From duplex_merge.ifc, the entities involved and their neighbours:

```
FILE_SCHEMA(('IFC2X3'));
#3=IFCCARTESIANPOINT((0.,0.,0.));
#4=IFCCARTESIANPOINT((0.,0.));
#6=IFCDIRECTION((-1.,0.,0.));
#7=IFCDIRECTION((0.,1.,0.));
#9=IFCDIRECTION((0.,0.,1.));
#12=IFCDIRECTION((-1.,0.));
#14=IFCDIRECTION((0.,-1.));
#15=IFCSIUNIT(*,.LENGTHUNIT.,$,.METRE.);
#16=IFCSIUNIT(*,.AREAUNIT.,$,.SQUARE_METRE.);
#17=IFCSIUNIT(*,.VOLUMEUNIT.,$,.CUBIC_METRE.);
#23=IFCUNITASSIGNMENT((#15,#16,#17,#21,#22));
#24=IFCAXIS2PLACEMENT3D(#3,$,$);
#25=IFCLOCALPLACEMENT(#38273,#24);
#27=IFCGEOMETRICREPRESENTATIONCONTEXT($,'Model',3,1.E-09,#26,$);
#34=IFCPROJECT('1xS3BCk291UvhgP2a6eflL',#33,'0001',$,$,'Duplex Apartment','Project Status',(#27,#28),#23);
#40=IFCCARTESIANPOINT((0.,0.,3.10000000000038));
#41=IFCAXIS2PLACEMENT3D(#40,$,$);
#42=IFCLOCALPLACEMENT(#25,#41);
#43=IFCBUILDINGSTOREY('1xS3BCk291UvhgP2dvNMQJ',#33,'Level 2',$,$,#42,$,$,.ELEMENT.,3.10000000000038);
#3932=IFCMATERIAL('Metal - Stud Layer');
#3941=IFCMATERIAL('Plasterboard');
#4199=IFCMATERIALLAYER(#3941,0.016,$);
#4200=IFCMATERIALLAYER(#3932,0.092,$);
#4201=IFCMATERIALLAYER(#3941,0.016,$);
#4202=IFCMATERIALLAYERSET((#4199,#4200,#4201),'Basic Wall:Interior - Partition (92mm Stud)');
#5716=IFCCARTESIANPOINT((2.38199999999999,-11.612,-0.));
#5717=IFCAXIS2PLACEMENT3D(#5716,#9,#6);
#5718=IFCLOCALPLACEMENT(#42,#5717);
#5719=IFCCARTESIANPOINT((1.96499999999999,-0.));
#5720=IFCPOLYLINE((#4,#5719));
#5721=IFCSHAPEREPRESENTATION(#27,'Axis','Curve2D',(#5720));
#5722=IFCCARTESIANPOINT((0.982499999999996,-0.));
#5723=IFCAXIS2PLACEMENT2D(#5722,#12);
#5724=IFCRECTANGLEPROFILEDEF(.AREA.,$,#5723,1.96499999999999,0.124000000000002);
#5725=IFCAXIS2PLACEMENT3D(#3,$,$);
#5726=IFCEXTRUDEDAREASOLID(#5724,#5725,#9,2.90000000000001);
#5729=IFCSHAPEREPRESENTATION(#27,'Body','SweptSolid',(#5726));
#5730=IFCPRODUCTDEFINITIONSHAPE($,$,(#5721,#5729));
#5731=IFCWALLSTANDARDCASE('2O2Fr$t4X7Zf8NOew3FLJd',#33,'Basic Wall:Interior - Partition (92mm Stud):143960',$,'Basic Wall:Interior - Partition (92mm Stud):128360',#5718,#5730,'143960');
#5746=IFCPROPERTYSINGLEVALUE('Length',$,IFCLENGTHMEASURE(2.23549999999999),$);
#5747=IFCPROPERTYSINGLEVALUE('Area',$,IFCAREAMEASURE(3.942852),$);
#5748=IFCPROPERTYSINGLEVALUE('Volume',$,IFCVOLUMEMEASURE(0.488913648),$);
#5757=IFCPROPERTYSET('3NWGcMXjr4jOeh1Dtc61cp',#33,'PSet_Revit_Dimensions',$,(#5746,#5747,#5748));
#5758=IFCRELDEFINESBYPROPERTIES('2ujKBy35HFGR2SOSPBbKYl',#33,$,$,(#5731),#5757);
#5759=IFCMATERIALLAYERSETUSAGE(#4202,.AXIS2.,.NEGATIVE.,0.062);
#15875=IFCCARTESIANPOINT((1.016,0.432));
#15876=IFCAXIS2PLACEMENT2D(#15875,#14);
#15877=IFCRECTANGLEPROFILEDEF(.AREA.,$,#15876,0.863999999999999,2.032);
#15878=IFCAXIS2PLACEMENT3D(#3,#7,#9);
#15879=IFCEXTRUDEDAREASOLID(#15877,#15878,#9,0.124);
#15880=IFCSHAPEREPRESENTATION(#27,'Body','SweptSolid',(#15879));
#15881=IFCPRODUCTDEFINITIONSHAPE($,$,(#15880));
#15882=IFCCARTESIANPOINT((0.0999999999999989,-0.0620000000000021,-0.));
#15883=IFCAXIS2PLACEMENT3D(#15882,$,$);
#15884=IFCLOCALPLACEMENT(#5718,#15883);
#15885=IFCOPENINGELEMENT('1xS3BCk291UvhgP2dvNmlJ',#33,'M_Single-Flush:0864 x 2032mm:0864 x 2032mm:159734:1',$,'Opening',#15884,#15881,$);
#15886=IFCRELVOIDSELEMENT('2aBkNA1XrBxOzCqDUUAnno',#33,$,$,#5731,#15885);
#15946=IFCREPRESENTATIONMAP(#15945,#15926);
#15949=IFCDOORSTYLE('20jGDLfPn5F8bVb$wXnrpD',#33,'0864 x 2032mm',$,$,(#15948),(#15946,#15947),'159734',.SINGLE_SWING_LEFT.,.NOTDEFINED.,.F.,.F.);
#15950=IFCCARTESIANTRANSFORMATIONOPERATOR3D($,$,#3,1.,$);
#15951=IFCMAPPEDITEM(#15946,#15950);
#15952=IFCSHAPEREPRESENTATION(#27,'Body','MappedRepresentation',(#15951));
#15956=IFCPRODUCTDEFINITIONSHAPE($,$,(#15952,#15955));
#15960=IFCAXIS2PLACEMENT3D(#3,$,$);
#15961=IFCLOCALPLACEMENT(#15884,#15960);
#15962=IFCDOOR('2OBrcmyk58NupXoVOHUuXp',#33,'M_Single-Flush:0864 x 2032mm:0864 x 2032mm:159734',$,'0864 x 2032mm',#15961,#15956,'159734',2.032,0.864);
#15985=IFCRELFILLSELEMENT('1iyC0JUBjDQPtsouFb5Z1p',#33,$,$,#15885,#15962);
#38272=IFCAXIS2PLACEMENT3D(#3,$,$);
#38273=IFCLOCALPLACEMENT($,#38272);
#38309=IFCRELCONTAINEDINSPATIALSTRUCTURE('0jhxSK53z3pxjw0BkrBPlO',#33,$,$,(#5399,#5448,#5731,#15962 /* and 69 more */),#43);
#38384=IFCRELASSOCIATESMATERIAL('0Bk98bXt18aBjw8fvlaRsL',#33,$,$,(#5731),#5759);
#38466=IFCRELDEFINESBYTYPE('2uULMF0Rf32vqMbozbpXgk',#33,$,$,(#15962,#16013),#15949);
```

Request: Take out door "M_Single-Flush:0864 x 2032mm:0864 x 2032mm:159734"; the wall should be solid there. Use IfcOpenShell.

```python
import ifcopenshell
import ifcopenshell.api.feature
import ifcopenshell.api.pset
import ifcopenshell.api.root
import ifcopenshell.geom
import ifcopenshell.util.element
import ifcopenshell.util.shape
import ifcopenshell.util.unit

model = ifcopenshell.open("duplex_merge.ifc")
area_scale = ifcopenshell.util.unit.calculate_unit_scale(model, "AREAUNIT")
volume_scale = ifcopenshell.util.unit.calculate_unit_scale(model, "VOLUMEUNIT")
settings = ifcopenshell.geom.settings()


def volume(element):
    """Net volume in cubic metres, openings subtracted."""
    shape = ifcopenshell.geom.create_shape(settings, element)
    return ifcopenshell.util.shape.get_volume(shape.geometry)


door = model.by_id(15962)
opening = door.FillsVoids[0].RelatingOpeningElement
wall = opening.VoidsElements[0].RelatingBuildingElement
before = volume(wall)

ifcopenshell.api.root.remove_product(model, product=door)
ifcopenshell.api.feature.remove_feature(model, feature=opening)

after = volume(wall)
thickness = 0.124  # wall thickness in metres

# Update the wall's stored quantities.
pset = model.by_id(ifcopenshell.util.element.get_pset(wall, "PSet_Revit_Dimensions", should_inherit=False)["id"])
ifcopenshell.api.pset.edit_pset(model, pset=pset, properties={
    "Area": model.create_entity("IfcAreaMeasure", after / thickness / area_scale),
    "Volume": model.create_entity("IfcVolumeMeasure", after / volume_scale),
})

print(f"wall volume {before:.3f} -> {after:.3f} m3")

model.write("duplex_merge_v2.ifc")
```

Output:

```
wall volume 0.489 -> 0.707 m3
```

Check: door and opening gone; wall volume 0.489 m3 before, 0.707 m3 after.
